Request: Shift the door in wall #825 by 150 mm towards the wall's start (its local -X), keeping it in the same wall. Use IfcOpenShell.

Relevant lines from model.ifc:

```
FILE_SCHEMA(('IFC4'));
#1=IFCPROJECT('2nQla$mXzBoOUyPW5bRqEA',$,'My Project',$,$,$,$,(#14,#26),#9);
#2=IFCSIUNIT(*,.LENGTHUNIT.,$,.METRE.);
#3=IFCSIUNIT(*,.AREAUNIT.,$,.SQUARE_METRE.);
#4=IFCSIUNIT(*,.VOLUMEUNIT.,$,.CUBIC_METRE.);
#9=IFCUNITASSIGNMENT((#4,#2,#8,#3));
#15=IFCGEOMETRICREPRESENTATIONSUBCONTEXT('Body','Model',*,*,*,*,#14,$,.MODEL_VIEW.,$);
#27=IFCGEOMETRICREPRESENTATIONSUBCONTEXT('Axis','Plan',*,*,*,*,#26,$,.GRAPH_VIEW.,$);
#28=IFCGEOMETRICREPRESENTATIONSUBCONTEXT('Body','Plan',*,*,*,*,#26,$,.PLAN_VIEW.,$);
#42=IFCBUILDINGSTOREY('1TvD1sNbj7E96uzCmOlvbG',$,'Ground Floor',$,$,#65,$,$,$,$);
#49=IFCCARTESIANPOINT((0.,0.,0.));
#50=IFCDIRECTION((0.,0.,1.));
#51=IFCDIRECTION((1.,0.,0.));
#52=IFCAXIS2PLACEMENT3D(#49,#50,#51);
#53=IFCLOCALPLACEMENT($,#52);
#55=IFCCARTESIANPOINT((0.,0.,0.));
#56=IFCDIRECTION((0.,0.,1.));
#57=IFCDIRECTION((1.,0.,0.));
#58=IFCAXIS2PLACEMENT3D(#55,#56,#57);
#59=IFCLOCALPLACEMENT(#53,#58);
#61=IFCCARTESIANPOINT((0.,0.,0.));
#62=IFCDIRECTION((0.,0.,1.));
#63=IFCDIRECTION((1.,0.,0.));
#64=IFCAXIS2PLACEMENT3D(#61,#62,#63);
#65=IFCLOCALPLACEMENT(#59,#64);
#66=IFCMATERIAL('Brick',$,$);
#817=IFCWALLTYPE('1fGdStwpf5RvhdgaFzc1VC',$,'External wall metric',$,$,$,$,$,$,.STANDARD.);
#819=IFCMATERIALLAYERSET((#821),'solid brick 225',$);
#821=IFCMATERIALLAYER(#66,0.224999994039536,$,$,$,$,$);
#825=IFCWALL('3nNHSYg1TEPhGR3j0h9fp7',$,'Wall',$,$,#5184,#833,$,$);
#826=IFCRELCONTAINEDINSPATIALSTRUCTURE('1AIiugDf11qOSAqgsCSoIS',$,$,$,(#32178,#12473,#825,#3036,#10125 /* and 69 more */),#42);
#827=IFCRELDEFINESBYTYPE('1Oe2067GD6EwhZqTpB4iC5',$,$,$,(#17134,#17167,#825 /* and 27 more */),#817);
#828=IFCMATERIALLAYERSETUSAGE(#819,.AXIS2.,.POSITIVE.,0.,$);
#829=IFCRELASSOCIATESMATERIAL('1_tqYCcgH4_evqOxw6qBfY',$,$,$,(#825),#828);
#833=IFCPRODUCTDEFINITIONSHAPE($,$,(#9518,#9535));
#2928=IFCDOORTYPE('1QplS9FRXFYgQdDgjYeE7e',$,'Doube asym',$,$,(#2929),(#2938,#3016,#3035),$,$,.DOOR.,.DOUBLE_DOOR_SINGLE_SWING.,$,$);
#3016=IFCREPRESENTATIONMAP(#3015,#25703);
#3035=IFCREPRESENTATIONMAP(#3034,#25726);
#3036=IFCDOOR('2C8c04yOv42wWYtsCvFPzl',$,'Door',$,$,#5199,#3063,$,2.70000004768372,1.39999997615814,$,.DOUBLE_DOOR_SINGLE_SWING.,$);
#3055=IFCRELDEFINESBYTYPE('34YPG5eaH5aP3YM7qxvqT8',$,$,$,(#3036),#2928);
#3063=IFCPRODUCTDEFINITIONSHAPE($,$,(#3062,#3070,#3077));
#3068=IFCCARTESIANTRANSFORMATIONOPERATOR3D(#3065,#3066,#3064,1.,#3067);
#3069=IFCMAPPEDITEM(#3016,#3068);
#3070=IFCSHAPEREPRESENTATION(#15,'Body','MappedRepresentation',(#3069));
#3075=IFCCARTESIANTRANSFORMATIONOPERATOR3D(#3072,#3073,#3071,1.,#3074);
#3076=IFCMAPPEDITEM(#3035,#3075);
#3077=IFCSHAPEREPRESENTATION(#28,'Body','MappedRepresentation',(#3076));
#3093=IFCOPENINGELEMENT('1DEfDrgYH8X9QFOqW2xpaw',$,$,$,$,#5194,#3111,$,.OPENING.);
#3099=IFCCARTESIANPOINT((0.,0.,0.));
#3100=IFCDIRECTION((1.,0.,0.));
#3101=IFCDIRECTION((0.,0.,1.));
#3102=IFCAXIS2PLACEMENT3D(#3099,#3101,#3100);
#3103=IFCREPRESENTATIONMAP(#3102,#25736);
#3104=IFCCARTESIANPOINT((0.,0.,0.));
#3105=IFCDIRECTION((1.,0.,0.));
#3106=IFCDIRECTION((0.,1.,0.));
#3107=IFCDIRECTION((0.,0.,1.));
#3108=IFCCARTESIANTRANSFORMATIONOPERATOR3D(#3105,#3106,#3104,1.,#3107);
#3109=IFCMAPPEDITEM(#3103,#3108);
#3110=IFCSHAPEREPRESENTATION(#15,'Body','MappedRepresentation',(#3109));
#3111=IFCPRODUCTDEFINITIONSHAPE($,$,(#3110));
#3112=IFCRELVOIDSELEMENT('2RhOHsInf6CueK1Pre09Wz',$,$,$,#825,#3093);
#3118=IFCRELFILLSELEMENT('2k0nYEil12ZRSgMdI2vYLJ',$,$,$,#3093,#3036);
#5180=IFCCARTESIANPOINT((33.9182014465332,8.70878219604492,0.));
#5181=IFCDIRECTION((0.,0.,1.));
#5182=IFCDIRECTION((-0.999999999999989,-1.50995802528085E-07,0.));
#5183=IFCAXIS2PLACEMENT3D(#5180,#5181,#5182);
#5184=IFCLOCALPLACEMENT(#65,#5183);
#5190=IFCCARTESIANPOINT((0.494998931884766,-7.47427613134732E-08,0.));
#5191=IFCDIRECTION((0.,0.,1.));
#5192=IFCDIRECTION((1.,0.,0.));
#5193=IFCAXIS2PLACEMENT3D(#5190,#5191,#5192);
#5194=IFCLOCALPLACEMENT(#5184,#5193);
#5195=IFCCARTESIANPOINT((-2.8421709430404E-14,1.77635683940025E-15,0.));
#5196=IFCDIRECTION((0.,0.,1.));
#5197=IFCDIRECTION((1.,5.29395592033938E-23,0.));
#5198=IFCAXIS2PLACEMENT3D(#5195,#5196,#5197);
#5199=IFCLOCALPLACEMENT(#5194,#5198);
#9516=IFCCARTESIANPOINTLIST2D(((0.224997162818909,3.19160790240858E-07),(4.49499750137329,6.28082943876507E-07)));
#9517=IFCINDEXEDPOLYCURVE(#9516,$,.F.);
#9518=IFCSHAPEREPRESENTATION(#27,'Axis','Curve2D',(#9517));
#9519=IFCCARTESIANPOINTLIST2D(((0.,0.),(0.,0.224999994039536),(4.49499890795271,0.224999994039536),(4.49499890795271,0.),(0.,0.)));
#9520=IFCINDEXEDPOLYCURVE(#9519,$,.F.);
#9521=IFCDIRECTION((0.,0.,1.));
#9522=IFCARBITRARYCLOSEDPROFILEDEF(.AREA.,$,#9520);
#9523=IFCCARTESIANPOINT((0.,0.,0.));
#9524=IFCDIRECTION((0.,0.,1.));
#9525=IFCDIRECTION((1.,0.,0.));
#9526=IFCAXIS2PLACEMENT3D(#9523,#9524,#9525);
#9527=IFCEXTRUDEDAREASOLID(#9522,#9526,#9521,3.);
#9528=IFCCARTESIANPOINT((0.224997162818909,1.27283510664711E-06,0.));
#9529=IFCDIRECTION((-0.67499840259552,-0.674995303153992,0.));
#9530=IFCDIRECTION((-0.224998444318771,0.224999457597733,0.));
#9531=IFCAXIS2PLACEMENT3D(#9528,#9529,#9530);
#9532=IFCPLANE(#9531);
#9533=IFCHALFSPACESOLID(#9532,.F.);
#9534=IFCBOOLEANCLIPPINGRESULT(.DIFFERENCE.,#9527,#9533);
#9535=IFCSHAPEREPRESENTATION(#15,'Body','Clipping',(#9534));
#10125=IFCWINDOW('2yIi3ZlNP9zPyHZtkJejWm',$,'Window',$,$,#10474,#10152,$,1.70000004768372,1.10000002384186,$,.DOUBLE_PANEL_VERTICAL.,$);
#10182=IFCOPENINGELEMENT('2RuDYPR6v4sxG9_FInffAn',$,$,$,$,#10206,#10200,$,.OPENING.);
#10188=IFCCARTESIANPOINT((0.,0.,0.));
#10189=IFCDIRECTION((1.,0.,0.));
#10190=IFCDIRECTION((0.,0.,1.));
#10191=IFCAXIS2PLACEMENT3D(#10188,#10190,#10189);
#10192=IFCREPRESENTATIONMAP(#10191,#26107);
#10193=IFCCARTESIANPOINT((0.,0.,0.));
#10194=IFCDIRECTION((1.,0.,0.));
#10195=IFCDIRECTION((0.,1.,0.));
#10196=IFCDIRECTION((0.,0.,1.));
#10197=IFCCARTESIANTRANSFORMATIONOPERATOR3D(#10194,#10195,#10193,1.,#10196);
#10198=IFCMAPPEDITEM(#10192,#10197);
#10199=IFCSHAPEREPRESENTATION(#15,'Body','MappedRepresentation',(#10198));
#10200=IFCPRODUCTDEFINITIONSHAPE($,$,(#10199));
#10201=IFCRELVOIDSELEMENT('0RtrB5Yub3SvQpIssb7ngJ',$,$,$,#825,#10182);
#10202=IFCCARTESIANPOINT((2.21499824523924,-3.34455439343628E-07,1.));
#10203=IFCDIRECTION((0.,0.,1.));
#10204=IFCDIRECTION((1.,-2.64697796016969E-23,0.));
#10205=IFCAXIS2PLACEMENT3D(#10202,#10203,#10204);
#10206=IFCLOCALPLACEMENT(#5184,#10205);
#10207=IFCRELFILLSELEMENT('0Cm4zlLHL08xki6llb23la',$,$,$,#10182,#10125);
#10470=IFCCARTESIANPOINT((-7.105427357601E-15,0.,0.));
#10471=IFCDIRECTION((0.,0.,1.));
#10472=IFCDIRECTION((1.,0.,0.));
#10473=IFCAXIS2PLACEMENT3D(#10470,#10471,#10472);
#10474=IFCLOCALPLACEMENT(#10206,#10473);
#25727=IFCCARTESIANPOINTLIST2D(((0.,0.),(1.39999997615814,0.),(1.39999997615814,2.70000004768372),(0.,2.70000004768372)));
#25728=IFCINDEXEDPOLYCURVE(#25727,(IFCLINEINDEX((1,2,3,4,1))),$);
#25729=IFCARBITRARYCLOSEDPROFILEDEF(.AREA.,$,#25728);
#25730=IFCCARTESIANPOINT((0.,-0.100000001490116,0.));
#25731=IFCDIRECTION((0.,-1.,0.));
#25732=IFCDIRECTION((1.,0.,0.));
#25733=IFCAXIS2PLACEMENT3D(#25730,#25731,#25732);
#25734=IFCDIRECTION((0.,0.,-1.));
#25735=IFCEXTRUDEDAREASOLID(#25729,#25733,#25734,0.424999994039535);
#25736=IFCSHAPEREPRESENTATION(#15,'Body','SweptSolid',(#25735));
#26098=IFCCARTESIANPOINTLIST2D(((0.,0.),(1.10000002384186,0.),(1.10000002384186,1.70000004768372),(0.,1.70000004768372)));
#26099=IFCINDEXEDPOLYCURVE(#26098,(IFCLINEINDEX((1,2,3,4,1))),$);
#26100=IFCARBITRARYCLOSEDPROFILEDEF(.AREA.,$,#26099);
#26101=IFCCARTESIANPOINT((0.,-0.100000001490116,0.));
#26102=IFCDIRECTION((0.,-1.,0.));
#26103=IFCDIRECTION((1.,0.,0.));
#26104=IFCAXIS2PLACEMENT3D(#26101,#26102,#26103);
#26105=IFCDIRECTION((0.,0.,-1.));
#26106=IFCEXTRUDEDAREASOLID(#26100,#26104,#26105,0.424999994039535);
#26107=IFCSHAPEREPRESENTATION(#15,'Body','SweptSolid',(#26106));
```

```python
import ifcopenshell
import ifcopenshell.api.geometry
import ifcopenshell.util.placement

model = ifcopenshell.open("model.ifc")

door = model.by_guid("2C8c04yOv42wWYtsCvFPzl")
opening = door.FillsVoids[0].RelatingOpeningElement
wall = opening.VoidsElements[0].RelatingBuildingElement

wall_matrix = ifcopenshell.util.placement.get_local_placement(wall.ObjectPlacement)
shift = wall_matrix[:3, 0] * -0.15
before = ifcopenshell.util.placement.get_local_placement(door.ObjectPlacement)[:3, 3].copy()

# The door is placed relative to its opening, so it follows when the opening moves.
matrix = ifcopenshell.util.placement.get_local_placement(opening.ObjectPlacement)
matrix[:3, 3] += shift
ifcopenshell.api.geometry.edit_object_placement(
    model, product=opening, matrix=matrix, is_si=False, should_transform_children=True
)

after = ifcopenshell.util.placement.get_local_placement(door.ObjectPlacement)[:3, 3]
print("door moved by", (after - before).round(3) + 0.0)

model.write("model_v2.ifc")
```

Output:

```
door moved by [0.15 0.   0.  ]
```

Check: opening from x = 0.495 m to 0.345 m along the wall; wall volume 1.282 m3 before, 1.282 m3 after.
